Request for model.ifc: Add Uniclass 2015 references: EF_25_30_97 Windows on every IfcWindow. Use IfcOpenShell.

First a look at what the model holds.

```python
import ifcopenshell

model = ifcopenshell.open("model.ifc")
print(model.schema)
print("classifications:", [c.Name for c in model.by_type("IfcClassification")])
for ifc_class in ("IfcDoor", "IfcRoof", "IfcStair", "IfcWall", "IfcWindow"):
    print(ifc_class, len(model.by_type(ifc_class)))
```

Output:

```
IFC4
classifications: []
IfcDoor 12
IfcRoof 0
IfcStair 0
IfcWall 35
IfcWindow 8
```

```python
import ifcopenshell
import ifcopenshell.api.classification

model = ifcopenshell.open("model.ifc")

system = ifcopenshell.api.classification.add_classification(model, classification="Uniclass 2015")

codes = {
    "IfcWindow": ("EF_25_30_97", "Windows"),
}
for ifc_class, (code, name) in codes.items():
    products = model.by_type(ifc_class)
    ifcopenshell.api.classification.add_reference(
        model, products=products, classification=system, identification=code, name=name
    )
    print(code, len(products))

model.write("model_v2.ifc")
```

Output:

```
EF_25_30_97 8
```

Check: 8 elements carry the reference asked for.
